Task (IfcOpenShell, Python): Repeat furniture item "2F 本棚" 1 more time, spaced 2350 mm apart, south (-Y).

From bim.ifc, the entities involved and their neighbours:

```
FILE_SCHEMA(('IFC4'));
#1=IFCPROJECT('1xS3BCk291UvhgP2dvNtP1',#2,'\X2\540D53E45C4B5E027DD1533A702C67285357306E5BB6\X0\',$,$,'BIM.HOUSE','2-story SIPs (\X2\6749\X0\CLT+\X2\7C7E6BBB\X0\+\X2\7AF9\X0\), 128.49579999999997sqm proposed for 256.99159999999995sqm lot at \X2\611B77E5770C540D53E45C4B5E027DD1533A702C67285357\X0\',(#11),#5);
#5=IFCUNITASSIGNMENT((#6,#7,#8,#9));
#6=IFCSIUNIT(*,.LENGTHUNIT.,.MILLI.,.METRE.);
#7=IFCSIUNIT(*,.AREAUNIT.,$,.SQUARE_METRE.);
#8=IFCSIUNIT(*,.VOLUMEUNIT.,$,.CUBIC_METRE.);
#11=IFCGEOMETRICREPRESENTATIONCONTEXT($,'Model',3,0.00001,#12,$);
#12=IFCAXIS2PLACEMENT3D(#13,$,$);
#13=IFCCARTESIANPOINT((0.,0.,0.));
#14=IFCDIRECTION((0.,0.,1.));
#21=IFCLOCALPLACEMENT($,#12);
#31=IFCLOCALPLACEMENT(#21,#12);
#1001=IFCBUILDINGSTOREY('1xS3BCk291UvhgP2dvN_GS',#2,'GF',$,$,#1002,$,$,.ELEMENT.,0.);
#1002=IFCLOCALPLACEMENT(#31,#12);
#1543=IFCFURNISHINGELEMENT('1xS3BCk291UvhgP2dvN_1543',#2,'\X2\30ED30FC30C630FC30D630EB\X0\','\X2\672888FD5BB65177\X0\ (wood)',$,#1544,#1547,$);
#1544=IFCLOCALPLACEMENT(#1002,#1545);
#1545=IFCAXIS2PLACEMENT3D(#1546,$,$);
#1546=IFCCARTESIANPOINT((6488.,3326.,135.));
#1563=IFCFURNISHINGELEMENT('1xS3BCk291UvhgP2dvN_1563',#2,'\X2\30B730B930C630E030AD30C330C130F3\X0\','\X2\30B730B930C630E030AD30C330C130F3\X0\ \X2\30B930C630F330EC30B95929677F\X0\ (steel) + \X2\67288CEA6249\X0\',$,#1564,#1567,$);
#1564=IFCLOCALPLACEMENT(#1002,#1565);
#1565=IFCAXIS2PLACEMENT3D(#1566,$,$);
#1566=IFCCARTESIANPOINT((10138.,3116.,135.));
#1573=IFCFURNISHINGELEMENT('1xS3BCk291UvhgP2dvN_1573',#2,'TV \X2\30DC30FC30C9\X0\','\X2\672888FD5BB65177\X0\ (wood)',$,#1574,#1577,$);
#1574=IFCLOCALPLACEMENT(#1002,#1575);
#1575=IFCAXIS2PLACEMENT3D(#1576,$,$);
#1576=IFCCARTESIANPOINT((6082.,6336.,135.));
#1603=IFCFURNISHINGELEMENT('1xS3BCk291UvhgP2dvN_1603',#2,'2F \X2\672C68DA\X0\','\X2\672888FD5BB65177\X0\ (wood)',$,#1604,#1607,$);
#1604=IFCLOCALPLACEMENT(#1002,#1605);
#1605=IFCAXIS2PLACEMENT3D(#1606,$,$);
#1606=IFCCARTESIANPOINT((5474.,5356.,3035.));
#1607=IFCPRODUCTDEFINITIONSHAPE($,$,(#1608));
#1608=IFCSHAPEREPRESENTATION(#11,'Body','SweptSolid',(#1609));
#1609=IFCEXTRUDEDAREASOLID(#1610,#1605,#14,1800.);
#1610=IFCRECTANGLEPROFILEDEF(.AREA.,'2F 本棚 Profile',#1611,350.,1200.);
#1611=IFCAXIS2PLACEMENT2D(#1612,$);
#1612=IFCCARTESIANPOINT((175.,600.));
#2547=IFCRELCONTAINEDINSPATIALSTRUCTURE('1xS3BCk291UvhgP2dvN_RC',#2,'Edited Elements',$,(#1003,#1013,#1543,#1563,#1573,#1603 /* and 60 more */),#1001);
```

```python
import numpy as np
import ifcopenshell
import ifcopenshell.api.geometry
import ifcopenshell.api.root
import ifcopenshell.util.element
import ifcopenshell.util.placement

model = ifcopenshell.open("bim.ifc")


def reuse_history(source, copy):
    """copy_class also copies each property set's owner history, people and application; keep the originals."""
    for rel in copy.IsDefinedBy:
        if rel.is_a("IfcRelDefinesByProperties") and (history := rel.RelatingPropertyDefinition.OwnerHistory):
            rel.RelatingPropertyDefinition.OwnerHistory = source.OwnerHistory
            ifcopenshell.util.element.remove_deep2(model, history)


source = model.by_id(1603)
base = ifcopenshell.util.placement.get_local_placement(source.ObjectPlacement)
step = np.array([0.0, -1.0, 0.0]) * 2350.0

for i in range(1, 2):
    copy = ifcopenshell.api.root.copy_class(model, product=source)
    copy.Representation = ifcopenshell.util.element.copy_deep(
        model, source.Representation, exclude=["IfcGeometricRepresentationContext", "IfcRepresentationMap"]
    )
    reuse_history(source, copy)
    matrix = base.copy()
    matrix[:3, 3] += i * step
    print("added at", matrix[:3, 3].round(3) + 0.0)
    ifcopenshell.api.geometry.edit_object_placement(model, product=copy, matrix=matrix, is_si=False)

model.write("bim_rev.ifc")
```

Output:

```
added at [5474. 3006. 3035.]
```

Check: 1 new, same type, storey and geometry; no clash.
